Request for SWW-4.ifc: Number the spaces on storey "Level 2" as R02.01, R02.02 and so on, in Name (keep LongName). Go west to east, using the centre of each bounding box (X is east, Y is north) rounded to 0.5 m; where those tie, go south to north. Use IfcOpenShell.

First a look at what the model holds.

```python
import ifcopenshell
import ifcopenshell.util.element
import ifcopenshell.util.placement

model = ifcopenshell.open("SWW-4.ifc")
print(model.schema)
storey = next(s for s in model.by_type("IfcBuildingStorey") if s.Name == "Level 2")
spaces = [e for e in ifcopenshell.util.element.get_decomposition(storey) if e.is_a("IfcSpace")]
for e in sorted(spaces, key=lambda e: e.id()):
    origin = ifcopenshell.util.placement.get_local_placement(e.ObjectPlacement)[:3, 3]
    print(e.id(), e.Name, e.LongName, origin.round(2) + 0.0, sep=" | ")
```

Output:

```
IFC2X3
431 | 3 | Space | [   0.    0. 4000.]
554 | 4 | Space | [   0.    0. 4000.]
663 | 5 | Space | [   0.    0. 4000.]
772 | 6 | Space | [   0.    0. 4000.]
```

```python
import ifcopenshell
import ifcopenshell.geom
import ifcopenshell.util.element
import ifcopenshell.util.shape

model = ifcopenshell.open("SWW-4.ifc")
settings = ifcopenshell.geom.settings()
settings.set("use-world-coords", True)


def centre(element):
    shape = ifcopenshell.geom.create_shape(settings, element)
    return ifcopenshell.util.shape.get_bbox_centroid(shape.geometry)


storey = next(s for s in model.by_type("IfcBuildingStorey") if s.Name == "Level 2")
spaces = [e for e in ifcopenshell.util.element.get_decomposition(storey) if e.is_a("IfcSpace")]

# Insertion points can sit at a corner or the storey origin, so sort by the geometry (in metres).
centres = {e: centre(e) for e in spaces}
spaces.sort(key=lambda e: (round(centres[e][0] / 0.5), centres[e][1]))

for i, e in enumerate(spaces, start=1):
    number = f"R02.{i:02d}"
    e.Name = number
    print(e.id(), number)

model.write("SWW-4_v2.ifc")
```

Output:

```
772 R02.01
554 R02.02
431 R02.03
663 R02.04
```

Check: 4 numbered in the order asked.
